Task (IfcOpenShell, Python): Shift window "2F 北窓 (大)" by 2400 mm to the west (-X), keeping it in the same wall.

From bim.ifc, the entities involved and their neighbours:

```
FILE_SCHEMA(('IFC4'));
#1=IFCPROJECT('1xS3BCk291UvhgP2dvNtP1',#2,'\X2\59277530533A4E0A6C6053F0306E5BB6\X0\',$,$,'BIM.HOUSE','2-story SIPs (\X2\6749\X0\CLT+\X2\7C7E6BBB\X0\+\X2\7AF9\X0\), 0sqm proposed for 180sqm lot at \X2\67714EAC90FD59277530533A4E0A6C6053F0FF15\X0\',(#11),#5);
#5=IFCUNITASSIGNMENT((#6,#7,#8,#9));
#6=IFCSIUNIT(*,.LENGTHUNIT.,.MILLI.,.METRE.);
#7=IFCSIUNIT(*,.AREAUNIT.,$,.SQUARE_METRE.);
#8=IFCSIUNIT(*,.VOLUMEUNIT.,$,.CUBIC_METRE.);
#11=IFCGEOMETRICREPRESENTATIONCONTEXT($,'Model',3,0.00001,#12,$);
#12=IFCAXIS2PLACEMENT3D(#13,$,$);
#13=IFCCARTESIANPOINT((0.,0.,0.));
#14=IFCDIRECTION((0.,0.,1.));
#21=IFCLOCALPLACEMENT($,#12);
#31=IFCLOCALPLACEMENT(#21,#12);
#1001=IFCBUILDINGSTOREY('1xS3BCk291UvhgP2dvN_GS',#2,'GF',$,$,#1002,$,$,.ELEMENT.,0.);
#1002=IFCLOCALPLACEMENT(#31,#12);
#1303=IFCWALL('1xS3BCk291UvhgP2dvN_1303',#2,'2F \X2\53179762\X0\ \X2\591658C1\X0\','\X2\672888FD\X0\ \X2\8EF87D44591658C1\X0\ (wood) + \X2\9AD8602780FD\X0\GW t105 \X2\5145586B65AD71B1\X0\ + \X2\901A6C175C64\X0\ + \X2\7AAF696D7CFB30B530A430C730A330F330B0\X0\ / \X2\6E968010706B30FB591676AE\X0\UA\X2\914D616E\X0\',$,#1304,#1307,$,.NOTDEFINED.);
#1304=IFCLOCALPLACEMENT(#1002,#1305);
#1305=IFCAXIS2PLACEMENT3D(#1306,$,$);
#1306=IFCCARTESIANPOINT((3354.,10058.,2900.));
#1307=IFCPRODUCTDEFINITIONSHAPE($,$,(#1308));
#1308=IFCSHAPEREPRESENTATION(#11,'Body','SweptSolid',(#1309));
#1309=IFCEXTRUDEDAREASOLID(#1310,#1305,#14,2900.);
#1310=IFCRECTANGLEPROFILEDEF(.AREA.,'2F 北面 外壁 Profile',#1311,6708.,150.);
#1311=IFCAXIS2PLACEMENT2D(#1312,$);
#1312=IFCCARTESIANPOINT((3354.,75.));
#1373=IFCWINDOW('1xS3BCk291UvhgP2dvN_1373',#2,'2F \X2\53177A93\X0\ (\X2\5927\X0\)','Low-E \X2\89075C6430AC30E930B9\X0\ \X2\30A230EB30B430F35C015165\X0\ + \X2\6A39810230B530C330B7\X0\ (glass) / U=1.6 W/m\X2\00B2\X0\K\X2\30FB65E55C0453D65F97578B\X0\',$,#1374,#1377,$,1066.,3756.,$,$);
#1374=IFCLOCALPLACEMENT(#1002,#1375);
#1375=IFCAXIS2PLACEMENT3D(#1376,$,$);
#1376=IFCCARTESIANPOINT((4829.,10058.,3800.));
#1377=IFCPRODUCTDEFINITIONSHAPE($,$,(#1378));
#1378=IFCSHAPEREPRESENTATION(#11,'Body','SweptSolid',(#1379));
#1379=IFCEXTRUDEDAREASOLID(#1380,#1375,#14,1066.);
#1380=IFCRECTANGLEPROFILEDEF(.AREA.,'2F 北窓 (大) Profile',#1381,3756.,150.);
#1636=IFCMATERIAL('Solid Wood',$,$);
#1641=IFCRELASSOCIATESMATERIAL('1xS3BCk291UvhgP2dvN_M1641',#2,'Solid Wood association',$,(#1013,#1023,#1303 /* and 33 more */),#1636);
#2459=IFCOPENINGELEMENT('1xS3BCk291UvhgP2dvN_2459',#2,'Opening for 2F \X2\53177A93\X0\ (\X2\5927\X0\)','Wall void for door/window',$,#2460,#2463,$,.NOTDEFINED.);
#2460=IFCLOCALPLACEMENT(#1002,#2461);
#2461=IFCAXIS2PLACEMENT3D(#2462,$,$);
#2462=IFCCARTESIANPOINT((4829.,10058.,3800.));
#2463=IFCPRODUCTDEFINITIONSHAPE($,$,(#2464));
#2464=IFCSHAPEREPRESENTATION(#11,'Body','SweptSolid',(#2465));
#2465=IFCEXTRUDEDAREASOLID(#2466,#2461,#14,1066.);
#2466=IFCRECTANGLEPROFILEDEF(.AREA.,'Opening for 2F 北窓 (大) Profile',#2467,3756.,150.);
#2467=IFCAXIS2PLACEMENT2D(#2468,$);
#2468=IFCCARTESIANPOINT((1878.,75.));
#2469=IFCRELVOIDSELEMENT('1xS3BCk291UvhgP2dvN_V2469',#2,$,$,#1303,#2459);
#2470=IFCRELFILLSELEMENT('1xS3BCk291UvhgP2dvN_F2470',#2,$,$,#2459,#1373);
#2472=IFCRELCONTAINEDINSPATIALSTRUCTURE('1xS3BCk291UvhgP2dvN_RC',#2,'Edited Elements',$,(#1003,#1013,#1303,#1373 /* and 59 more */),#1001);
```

```python
import ifcopenshell
import ifcopenshell.api.geometry
import ifcopenshell.util.placement

model = ifcopenshell.open("bim.ifc")

window = model.by_guid("1xS3BCk291UvhgP2dvN_1373")
opening = window.FillsVoids[0].RelatingOpeningElement
wall = opening.VoidsElements[0].RelatingBuildingElement

wall_matrix = ifcopenshell.util.placement.get_local_placement(wall.ObjectPlacement)
shift = wall_matrix[:3, 0] * -2400.0
before = ifcopenshell.util.placement.get_local_placement(window.ObjectPlacement)[:3, 3].copy()

# The window is not placed relative to its opening, so move both.
for product in (opening, window):
    matrix = ifcopenshell.util.placement.get_local_placement(product.ObjectPlacement)
    matrix[:3, 3] += shift
    ifcopenshell.api.geometry.edit_object_placement(model, product=product, matrix=matrix, is_si=False)

after = ifcopenshell.util.placement.get_local_placement(window.ObjectPlacement)[:3, 3]
print("window moved by", (after - before).round(3) + 0.0)

model.write("bim_rev.ifc")
```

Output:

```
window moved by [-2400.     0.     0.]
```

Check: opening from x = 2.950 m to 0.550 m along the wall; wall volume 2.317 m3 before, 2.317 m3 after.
